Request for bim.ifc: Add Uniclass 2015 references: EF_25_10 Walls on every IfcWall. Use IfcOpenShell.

First a look at what the model holds.

```python
import ifcopenshell

model = ifcopenshell.open("bim.ifc")
print(model.schema)
print("classifications:", [c.Name for c in model.by_type("IfcClassification")])
for ifc_class in ("IfcDoor", "IfcRoof", "IfcStair", "IfcWall", "IfcWindow"):
    print(ifc_class, len(model.by_type(ifc_class)))
```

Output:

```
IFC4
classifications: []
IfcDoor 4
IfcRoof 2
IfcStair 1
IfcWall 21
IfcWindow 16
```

```python
import ifcopenshell
import ifcopenshell.api.classification

model = ifcopenshell.open("bim.ifc")

system = ifcopenshell.api.classification.add_classification(model, classification="Uniclass 2015")

codes = {
    "IfcWall": ("EF_25_10", "Walls"),
}
for ifc_class, (code, name) in codes.items():
    products = model.by_type(ifc_class)
    ifcopenshell.api.classification.add_reference(
        model, products=products, classification=system, identification=code, name=name
    )
    print(code, len(products))

model.write("bim_rev.ifc")
```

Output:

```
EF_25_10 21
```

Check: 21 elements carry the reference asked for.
